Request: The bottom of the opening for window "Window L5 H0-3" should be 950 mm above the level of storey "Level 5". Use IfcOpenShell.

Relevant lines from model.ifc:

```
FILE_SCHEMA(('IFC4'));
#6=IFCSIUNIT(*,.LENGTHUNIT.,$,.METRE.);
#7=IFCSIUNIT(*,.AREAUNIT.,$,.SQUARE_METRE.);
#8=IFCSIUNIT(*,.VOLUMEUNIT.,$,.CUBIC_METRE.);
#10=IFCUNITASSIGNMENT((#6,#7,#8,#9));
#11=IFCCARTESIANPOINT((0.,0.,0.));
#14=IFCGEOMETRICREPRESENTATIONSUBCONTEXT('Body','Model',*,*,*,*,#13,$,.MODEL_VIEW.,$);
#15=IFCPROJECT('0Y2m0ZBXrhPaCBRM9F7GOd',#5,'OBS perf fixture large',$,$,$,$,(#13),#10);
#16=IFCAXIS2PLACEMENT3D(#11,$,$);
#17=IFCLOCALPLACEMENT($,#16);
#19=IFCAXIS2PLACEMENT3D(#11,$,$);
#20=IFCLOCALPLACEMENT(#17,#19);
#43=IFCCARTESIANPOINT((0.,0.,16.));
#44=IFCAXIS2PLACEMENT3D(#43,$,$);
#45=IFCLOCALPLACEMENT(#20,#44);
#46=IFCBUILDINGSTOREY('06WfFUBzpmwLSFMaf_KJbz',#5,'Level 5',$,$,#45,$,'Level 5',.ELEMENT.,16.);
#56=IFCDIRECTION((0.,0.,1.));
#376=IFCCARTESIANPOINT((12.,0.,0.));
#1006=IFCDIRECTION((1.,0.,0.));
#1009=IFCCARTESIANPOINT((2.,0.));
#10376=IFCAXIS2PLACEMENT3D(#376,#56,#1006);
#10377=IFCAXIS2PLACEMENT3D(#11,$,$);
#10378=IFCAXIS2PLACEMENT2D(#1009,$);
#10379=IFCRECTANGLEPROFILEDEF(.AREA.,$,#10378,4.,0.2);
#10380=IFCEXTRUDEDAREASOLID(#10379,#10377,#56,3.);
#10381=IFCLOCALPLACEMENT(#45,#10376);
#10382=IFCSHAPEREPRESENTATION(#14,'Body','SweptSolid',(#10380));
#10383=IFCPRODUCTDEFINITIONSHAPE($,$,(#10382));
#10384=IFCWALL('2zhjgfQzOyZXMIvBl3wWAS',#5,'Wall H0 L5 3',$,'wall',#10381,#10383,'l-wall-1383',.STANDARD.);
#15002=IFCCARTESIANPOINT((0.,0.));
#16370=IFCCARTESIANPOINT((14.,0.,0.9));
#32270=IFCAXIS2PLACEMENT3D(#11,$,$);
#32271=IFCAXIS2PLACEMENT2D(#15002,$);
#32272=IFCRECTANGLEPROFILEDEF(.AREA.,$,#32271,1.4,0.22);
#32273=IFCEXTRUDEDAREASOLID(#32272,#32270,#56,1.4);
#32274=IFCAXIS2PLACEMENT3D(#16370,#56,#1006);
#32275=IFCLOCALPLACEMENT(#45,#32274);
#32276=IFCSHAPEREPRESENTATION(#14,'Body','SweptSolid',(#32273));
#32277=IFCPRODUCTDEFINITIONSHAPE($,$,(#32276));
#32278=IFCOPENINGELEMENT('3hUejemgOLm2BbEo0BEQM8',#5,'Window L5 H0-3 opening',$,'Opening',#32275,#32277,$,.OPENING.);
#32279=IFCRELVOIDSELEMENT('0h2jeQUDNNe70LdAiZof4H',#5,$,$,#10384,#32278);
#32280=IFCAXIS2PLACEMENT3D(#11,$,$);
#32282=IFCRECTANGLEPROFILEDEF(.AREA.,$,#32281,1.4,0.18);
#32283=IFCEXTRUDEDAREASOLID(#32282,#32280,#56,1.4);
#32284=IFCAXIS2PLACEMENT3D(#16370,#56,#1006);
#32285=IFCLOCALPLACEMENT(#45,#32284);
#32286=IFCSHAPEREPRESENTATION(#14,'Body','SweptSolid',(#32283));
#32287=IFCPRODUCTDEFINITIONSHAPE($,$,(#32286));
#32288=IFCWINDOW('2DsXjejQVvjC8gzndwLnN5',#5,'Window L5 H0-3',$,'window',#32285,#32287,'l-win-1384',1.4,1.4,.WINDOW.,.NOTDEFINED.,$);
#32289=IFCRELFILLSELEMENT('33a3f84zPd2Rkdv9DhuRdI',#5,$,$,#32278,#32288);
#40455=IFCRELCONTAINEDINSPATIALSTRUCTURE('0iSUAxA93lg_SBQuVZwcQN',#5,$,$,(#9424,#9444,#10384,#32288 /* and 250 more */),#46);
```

```python
import numpy as np
import ifcopenshell
import ifcopenshell.api.geometry
import ifcopenshell.geom
import ifcopenshell.util.element
import ifcopenshell.util.placement
import ifcopenshell.util.shape
import ifcopenshell.util.unit

model = ifcopenshell.open("model.ifc")
unit_scale = ifcopenshell.util.unit.calculate_unit_scale(model)

window = model.by_guid("2DsXjejQVvjC8gzndwLnN5")
opening = window.FillsVoids[0].RelatingOpeningElement
storey = ifcopenshell.util.element.get_container(window, ifc_class="IfcBuildingStorey")
level = ifcopenshell.util.placement.get_local_placement(storey.ObjectPlacement)[2, 3]

# The opening's origin need not be at the sill, so measure its lowest point.
shape = ifcopenshell.geom.create_shape(ifcopenshell.geom.settings(), opening)
bottom = ifcopenshell.util.shape.get_shape_bottom_elevation(shape, shape.geometry) / unit_scale
dz = level + 0.95 / unit_scale - bottom

shift = np.array([0.0, 0.0, dz])
# The window is not placed relative to its opening, so move both.
for product in (opening, window):
    matrix = ifcopenshell.util.placement.get_local_placement(product.ObjectPlacement)
    matrix[:3, 3] += shift
    ifcopenshell.api.geometry.edit_object_placement(model, product=product, matrix=matrix, is_si=False)

print(f"moved by {dz * unit_scale:+.3f} m")

model.write("model_rev.ifc")
```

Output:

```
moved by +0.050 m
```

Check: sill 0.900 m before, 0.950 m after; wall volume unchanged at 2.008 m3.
